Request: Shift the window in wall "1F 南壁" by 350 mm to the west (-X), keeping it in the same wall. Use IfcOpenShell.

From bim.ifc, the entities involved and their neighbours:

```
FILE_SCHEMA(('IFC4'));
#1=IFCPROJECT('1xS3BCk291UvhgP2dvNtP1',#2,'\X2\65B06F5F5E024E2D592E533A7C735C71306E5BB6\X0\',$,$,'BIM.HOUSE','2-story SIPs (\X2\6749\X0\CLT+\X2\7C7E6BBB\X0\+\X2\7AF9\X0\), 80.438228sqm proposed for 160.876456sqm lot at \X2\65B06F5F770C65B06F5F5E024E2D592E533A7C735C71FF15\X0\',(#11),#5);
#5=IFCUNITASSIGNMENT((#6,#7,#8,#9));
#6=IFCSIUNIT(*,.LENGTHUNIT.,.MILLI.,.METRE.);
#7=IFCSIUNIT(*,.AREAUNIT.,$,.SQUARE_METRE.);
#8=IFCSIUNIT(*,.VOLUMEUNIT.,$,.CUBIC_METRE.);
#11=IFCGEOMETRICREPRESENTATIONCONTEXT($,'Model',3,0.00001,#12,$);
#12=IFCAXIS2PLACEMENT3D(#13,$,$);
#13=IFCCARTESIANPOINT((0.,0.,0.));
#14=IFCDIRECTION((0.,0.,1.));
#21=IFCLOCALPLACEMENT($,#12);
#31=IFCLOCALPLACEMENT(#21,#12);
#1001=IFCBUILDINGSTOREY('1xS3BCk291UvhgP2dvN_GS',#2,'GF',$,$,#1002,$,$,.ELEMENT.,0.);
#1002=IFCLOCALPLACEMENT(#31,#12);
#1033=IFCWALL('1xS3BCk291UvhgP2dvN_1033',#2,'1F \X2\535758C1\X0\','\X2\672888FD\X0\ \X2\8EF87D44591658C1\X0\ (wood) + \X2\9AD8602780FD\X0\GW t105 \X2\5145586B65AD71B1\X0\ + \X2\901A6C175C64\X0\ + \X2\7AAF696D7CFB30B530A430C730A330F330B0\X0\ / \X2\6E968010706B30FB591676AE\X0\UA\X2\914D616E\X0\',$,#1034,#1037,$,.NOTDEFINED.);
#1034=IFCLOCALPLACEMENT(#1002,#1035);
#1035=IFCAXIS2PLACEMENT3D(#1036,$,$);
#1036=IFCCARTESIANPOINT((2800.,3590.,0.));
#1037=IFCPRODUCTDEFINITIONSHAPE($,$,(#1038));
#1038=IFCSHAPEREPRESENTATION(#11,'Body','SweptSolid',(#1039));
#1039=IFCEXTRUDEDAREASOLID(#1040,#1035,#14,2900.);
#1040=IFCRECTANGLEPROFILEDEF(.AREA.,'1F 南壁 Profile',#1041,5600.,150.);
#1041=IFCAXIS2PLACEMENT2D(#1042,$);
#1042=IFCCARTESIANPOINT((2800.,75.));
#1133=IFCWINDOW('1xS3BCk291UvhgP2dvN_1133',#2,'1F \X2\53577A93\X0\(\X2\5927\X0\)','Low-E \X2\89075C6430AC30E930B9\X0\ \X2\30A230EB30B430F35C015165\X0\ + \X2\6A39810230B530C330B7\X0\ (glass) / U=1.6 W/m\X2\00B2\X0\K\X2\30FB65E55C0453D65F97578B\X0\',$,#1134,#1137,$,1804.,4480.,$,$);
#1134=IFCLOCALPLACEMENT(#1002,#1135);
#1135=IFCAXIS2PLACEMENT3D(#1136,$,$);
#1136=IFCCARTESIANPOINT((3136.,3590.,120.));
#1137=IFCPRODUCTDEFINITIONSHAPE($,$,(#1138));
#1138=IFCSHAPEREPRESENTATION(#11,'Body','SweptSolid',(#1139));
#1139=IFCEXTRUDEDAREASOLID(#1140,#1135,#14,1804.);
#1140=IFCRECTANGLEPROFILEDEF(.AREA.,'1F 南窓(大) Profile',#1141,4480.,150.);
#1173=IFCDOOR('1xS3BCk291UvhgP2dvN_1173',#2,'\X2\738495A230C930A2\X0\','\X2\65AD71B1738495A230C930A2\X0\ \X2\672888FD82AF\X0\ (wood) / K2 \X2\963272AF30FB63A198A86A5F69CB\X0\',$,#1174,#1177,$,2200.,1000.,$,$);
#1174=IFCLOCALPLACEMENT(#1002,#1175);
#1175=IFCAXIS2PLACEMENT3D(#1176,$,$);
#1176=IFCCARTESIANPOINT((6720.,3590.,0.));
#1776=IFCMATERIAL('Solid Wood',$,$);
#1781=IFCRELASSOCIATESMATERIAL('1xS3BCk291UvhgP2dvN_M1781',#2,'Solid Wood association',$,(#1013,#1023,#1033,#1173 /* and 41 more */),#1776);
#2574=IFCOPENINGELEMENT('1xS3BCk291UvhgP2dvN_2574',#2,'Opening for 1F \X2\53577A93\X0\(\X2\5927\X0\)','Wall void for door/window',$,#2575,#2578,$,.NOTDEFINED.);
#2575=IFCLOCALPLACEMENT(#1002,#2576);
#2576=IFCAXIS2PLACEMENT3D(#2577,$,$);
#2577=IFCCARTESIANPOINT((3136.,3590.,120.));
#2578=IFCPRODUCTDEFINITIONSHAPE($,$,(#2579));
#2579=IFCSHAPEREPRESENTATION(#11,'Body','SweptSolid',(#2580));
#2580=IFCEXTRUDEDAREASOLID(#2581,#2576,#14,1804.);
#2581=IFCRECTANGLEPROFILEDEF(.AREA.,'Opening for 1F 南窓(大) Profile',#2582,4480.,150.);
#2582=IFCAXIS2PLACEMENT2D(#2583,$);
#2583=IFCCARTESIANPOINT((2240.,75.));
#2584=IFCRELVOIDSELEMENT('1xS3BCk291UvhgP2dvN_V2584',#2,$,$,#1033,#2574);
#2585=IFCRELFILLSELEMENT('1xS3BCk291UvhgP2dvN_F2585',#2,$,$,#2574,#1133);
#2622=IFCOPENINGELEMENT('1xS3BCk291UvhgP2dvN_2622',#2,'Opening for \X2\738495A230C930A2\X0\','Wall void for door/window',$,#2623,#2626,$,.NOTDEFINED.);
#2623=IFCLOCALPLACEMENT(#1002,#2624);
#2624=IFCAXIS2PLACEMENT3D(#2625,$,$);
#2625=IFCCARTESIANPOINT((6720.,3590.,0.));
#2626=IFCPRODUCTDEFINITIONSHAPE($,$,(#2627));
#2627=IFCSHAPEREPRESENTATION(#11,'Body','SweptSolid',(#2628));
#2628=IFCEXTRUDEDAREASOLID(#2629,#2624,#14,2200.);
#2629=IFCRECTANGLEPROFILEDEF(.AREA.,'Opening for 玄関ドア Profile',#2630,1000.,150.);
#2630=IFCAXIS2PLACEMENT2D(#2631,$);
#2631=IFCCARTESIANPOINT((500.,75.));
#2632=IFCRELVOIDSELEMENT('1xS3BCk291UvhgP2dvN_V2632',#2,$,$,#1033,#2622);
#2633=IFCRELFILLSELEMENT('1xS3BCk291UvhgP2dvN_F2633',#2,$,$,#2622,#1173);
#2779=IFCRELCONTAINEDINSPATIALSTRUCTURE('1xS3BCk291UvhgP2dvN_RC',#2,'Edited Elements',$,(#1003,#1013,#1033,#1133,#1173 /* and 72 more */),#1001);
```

```python
import ifcopenshell
import ifcopenshell.api.geometry
import ifcopenshell.util.placement

model = ifcopenshell.open("bim.ifc")

window = model.by_id(1133)
opening = window.FillsVoids[0].RelatingOpeningElement
wall = opening.VoidsElements[0].RelatingBuildingElement

wall_matrix = ifcopenshell.util.placement.get_local_placement(wall.ObjectPlacement)
shift = wall_matrix[:3, 0] * -350.0
before = ifcopenshell.util.placement.get_local_placement(window.ObjectPlacement)[:3, 3].copy()

# The window is not placed relative to its opening, so move both.
for product in (opening, window):
    matrix = ifcopenshell.util.placement.get_local_placement(product.ObjectPlacement)
    matrix[:3, 3] += shift
    ifcopenshell.api.geometry.edit_object_placement(model, product=product, matrix=matrix, is_si=False)

after = ifcopenshell.util.placement.get_local_placement(window.ObjectPlacement)[:3, 3]
print("window moved by", (after - before).round(3) + 0.0)

model.write("bim-out.ifc")
```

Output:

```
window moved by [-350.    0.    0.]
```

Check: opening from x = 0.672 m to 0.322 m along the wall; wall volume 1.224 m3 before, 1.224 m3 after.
